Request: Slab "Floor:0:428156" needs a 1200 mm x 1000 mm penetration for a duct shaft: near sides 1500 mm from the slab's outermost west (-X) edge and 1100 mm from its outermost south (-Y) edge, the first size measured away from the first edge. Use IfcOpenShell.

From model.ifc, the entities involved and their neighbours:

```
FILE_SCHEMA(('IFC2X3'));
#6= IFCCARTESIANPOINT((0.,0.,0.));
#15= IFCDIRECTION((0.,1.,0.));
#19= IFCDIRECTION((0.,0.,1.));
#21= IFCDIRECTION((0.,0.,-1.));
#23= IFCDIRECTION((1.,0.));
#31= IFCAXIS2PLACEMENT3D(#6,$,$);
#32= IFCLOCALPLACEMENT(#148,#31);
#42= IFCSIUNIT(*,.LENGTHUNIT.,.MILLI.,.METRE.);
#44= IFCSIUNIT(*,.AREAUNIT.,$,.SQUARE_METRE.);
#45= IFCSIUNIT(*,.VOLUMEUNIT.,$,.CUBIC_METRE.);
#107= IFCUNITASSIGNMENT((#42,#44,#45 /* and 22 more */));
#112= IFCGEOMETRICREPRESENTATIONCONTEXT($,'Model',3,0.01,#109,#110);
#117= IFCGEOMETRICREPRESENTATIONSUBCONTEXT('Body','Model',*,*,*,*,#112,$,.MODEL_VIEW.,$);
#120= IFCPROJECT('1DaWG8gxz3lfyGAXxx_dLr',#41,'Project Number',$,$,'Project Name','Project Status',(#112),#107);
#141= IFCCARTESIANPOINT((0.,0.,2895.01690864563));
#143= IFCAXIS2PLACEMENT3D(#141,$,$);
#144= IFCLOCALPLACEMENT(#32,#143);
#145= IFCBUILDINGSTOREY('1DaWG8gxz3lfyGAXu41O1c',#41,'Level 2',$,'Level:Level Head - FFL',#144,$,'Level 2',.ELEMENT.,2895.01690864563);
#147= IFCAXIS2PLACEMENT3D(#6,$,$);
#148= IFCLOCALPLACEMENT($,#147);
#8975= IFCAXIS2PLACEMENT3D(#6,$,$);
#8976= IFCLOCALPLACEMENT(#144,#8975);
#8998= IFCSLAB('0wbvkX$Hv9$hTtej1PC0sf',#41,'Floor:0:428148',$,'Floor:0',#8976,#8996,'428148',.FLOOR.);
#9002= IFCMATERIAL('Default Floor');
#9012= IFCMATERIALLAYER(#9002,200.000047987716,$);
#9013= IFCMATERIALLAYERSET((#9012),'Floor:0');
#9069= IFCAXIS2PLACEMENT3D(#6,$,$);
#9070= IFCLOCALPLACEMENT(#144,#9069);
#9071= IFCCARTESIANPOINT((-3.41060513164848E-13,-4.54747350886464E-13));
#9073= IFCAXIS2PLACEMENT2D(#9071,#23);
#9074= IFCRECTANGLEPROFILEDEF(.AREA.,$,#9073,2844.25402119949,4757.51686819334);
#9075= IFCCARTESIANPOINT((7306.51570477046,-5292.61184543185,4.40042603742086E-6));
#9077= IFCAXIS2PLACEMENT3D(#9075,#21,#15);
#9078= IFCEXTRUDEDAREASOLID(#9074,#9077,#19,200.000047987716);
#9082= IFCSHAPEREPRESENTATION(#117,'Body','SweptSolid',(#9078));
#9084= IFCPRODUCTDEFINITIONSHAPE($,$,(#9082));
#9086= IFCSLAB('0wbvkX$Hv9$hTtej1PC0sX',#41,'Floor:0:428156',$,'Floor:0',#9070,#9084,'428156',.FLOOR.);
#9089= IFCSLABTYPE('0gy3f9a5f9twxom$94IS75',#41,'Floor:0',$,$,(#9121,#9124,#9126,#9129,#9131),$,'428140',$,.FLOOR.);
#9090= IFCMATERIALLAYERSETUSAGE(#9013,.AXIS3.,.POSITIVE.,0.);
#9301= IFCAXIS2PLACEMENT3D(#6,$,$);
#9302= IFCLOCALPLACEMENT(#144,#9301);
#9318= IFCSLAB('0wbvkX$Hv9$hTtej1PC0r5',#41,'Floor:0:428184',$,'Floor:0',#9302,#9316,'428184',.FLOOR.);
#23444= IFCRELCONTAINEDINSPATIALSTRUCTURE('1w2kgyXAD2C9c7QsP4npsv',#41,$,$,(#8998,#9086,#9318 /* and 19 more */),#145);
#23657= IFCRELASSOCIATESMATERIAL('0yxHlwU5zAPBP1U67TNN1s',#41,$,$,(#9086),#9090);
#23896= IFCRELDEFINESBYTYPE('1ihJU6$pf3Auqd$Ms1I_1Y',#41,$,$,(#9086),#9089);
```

```python
import numpy as np
import ifcopenshell
import ifcopenshell.api.feature
import ifcopenshell.api.geometry
import ifcopenshell.api.root
import ifcopenshell.geom
import ifcopenshell.util.placement
import ifcopenshell.util.representation
import ifcopenshell.util.shape
import ifcopenshell.util.unit

model = ifcopenshell.open("model.ifc")
unit_scale = ifcopenshell.util.unit.calculate_unit_scale(model)
settings = ifcopenshell.geom.settings()


def volume(element):
    """Net volume in cubic metres, openings subtracted."""
    shape = ifcopenshell.geom.create_shape(settings, element)
    return ifcopenshell.util.shape.get_volume(shape.geometry)


slab = model.by_id(9086)
before = volume(slab)

# Extent in the slab's own axes, in metres. The edges named are its -X and -Y sides.
slab_shape = ifcopenshell.geom.create_shape(settings, slab)
vertices = ifcopenshell.util.shape.get_vertices(slab_shape.geometry)
x_min, y_min, bottom = vertices.min(axis=0)
top = vertices[:, 2].max()

opening = ifcopenshell.api.root.create_entity(model, ifc_class="IfcOpeningElement", name="Duct shaft opening")
context = ifcopenshell.util.representation.get_context(model, "Model", "Body", "MODEL_VIEW")
width, depth = 1.2, 1
outline = [(0.0, 0.0), (width, 0.0), (width, depth), (0.0, depth), (0.0, 0.0)]
# Overshoot both faces by 50 mm so the cut is clean.
shape = ifcopenshell.api.geometry.add_slab_representation(
    model, context=context, depth=top - bottom + 0.1, polyline=outline
)
ifcopenshell.api.geometry.assign_representation(model, product=opening, representation=shape)

matrix = ifcopenshell.util.placement.get_local_placement(slab.ObjectPlacement)
matrix[:, 3] = matrix @ np.append(np.array([x_min + 1.5, y_min + 1.1, bottom - 0.05]) / unit_scale, 1.0)
ifcopenshell.api.geometry.edit_object_placement(model, product=opening, matrix=matrix, is_si=False)
ifcopenshell.api.feature.add_feature(model, feature=opening, element=slab)

after = volume(slab)

print(f"slab volume {before:.3f} -> {after:.3f} m3")

model.write("model_updated.ifc")
```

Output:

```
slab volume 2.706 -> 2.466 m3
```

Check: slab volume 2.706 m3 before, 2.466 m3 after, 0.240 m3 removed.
